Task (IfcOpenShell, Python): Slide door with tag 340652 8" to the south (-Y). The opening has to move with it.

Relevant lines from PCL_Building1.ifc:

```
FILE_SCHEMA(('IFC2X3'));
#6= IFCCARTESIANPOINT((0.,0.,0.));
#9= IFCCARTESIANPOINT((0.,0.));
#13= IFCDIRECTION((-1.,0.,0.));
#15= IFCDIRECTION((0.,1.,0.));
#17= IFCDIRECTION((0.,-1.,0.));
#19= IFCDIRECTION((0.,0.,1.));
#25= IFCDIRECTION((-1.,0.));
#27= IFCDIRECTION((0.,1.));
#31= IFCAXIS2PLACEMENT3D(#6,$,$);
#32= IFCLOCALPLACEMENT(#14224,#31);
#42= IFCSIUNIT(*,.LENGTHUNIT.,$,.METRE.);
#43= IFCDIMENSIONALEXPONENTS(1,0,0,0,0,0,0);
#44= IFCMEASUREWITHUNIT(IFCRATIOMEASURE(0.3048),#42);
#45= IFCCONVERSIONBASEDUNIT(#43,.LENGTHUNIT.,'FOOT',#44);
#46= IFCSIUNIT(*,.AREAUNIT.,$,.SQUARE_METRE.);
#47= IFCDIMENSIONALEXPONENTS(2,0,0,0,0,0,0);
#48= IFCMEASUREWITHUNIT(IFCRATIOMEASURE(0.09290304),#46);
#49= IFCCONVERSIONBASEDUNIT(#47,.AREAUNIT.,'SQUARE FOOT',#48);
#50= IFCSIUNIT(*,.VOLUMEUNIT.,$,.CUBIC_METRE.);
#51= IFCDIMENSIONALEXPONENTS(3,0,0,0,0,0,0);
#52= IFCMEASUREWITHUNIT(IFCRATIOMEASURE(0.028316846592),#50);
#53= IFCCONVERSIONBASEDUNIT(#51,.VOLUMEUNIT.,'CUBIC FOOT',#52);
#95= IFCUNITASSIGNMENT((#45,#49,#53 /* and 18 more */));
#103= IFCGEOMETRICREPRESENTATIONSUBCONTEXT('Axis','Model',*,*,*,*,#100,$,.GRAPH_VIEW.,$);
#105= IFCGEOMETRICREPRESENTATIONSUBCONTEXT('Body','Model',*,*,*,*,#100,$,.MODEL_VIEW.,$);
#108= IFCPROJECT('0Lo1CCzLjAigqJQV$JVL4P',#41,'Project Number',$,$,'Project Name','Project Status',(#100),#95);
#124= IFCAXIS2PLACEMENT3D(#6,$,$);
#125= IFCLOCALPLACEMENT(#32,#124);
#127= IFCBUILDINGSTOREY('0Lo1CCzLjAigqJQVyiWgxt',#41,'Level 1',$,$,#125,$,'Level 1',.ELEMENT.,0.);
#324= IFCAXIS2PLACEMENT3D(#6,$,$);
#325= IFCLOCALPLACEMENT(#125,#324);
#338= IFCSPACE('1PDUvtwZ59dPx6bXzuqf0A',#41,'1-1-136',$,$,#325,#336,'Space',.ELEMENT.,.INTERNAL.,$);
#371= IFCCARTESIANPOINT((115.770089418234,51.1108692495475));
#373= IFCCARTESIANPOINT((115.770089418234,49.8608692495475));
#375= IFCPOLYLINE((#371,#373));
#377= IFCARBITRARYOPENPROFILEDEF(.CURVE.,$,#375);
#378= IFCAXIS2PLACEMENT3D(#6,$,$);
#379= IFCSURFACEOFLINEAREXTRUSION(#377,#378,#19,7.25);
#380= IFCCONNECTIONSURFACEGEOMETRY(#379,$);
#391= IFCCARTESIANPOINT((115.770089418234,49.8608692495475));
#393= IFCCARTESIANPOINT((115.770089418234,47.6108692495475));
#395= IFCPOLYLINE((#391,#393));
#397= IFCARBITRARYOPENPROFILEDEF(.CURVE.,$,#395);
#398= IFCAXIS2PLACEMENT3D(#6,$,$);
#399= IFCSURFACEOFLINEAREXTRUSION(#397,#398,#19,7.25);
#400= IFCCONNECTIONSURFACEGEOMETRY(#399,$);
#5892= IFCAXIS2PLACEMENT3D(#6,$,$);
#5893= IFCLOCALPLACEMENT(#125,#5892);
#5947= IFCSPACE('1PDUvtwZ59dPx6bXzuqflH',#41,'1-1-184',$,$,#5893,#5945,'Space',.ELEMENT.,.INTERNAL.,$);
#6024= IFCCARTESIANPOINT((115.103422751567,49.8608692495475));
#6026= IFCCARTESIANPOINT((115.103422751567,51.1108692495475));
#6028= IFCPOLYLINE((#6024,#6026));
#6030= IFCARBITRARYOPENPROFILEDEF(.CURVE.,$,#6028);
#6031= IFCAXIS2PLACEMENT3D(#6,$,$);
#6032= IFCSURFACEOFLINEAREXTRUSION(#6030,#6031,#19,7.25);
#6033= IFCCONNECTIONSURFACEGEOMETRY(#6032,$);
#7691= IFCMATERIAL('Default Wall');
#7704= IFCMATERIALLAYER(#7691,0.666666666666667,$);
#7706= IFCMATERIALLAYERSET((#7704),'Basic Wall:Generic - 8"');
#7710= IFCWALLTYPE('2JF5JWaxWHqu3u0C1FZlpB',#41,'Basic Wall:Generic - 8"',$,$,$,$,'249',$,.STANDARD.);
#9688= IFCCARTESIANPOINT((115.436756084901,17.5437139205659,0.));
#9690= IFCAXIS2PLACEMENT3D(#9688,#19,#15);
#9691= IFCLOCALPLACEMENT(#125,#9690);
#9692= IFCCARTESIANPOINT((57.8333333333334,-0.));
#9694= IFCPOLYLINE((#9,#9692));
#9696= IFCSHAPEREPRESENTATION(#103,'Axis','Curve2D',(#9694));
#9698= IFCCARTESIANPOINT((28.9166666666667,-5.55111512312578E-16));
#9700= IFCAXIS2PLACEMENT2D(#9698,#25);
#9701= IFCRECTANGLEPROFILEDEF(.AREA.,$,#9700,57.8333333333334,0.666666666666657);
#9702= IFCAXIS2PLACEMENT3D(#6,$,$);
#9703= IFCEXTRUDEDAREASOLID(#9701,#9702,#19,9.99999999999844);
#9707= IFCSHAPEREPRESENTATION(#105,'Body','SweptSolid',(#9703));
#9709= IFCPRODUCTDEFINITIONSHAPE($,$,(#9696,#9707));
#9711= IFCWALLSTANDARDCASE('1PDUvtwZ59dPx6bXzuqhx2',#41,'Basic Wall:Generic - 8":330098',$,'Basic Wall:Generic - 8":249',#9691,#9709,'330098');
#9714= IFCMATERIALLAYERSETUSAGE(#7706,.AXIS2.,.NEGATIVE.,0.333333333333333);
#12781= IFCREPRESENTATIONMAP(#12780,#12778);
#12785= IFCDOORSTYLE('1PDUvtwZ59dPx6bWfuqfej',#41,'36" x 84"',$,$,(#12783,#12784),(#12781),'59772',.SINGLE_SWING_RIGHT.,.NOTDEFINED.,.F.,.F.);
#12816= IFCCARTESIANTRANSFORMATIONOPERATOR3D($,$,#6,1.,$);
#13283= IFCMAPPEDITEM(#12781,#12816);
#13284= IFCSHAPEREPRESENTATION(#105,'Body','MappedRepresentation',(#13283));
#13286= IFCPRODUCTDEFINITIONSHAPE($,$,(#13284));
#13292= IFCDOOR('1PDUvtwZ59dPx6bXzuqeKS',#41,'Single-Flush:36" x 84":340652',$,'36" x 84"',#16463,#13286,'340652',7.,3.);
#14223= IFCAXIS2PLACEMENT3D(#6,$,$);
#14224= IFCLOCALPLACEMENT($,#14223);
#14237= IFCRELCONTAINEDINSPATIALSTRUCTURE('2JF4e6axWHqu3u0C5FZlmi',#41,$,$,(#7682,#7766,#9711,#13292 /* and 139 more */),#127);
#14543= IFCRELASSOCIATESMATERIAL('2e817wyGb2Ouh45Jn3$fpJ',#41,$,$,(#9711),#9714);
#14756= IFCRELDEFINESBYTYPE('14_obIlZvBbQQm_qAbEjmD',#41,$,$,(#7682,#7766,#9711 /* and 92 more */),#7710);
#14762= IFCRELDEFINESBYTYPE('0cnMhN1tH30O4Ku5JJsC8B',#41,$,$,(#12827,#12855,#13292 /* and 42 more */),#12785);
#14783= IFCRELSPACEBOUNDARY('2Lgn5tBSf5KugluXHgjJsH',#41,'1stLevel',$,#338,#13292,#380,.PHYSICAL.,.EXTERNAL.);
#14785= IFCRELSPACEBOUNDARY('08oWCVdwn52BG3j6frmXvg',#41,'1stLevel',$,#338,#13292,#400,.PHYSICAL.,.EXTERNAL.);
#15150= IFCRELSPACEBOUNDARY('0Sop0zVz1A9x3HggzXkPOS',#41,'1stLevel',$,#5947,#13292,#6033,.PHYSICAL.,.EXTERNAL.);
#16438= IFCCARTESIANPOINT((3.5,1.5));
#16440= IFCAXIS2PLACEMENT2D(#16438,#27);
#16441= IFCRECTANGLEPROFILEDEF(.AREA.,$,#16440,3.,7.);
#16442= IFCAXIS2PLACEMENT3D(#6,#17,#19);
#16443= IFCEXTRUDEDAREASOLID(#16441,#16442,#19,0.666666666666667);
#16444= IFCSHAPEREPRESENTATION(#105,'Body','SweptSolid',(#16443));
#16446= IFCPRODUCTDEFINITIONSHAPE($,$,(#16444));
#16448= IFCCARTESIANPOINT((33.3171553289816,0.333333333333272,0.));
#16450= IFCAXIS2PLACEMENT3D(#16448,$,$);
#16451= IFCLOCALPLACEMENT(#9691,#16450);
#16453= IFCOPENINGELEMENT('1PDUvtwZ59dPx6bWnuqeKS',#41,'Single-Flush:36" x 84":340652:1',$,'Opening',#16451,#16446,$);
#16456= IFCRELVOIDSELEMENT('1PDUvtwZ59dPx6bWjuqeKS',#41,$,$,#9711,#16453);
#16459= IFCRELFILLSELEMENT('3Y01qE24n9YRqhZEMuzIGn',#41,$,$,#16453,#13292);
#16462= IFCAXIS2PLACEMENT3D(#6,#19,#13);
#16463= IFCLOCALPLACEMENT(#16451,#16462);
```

```python
import numpy as np
import ifcopenshell
import ifcopenshell.api.geometry
import ifcopenshell.util.placement
import ifcopenshell.util.unit

model = ifcopenshell.open("PCL_Building1.ifc")
unit_scale = ifcopenshell.util.unit.calculate_unit_scale(model)

door = model.by_id(13292)
opening = door.FillsVoids[0].RelatingOpeningElement
wall = opening.VoidsElements[0].RelatingBuildingElement

wall_matrix = ifcopenshell.util.placement.get_local_placement(wall.ObjectPlacement)
shift = wall_matrix[:3, 0] * -8 * 0.0254 / unit_scale
before = ifcopenshell.util.placement.get_local_placement(door.ObjectPlacement)[:3, 3].copy()

# The door is placed relative to its opening, so it follows when the opening moves.
matrix = ifcopenshell.util.placement.get_local_placement(opening.ObjectPlacement)
matrix[:3, 3] += shift
ifcopenshell.api.geometry.edit_object_placement(
    model, product=opening, matrix=matrix, is_si=False, should_transform_children=True
)

# Space boundary surfaces are stored in each space's coordinates; move them too.
for rel in door.ProvidesBoundaries:
    if not rel.ConnectionGeometry:
        continue
    surface = rel.ConnectionGeometry.SurfaceOnRelatingElement
    space_matrix = ifcopenshell.util.placement.get_local_placement(rel.RelatingSpace.ObjectPlacement)
    point = np.array(surface.Position.Location.Coordinates) + space_matrix[:3, :3].T @ shift
    surface.Position = model.createIfcAxis2Placement3D(
        model.createIfcCartesianPoint(point.tolist()), surface.Position.Axis, surface.Position.RefDirection
    )

after = ifcopenshell.util.placement.get_local_placement(door.ObjectPlacement)[:3, 3]
print("door moved by", (after - before).round(3) + 0.0)

model.write("PCL_Building1_updated.ifc")
```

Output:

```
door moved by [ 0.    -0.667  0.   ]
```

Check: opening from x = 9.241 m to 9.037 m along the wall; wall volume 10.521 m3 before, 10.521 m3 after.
